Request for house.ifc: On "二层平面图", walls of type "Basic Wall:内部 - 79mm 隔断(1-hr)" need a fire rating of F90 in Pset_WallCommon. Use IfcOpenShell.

First a look at what the model holds.

```python
import ifcopenshell
import ifcopenshell.util.element

model = ifcopenshell.open("house.ifc")
print(model.schema)
storey = next(s for s in model.by_type("IfcBuildingStorey") if s.Name == "二层平面图")
walls = [e for e in ifcopenshell.util.element.get_decomposition(storey) if e.is_a("IfcWall")]
seen = {}
for e in walls:
    element_type = ifcopenshell.util.element.get_type(e)
    key = (element_type.Name if element_type != e and element_type else None, ifcopenshell.util.element.get_pset(e, "Pset_WallCommon", "FireRating"))
    seen[key] = seen.get(key, 0) + 1
for (name, value), count in sorted(seen.items(), key=str):
    print(count, "x", name, "|", value)
```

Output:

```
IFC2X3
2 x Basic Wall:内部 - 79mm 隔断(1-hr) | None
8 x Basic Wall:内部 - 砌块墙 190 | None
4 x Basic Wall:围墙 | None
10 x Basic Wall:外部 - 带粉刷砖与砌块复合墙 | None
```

```python
import ifcopenshell
import ifcopenshell.api.pset
import ifcopenshell.util.element

model = ifcopenshell.open("house.ifc")

storey = next(s for s in model.by_type("IfcBuildingStorey") if s.Name == "二层平面图")
walls = [e for e in ifcopenshell.util.element.get_decomposition(storey) if e.is_a("IfcWall")]

count = 0
for e in walls:
    element_type = ifcopenshell.util.element.get_type(e)
    if element_type in (None, e) or element_type.Name != "Basic Wall:内部 - 79mm 隔断(1-hr)":
        continue
    # add_pset returns the element's existing set when there is one.
    pset = ifcopenshell.api.pset.add_pset(model, product=e, name="Pset_WallCommon")
    ifcopenshell.api.pset.edit_pset(model, pset=pset, properties={"FireRating": "F90"})
    count += 1

print(count, "walls updated")

model.write("house-out.ifc")
```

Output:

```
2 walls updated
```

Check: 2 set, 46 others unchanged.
